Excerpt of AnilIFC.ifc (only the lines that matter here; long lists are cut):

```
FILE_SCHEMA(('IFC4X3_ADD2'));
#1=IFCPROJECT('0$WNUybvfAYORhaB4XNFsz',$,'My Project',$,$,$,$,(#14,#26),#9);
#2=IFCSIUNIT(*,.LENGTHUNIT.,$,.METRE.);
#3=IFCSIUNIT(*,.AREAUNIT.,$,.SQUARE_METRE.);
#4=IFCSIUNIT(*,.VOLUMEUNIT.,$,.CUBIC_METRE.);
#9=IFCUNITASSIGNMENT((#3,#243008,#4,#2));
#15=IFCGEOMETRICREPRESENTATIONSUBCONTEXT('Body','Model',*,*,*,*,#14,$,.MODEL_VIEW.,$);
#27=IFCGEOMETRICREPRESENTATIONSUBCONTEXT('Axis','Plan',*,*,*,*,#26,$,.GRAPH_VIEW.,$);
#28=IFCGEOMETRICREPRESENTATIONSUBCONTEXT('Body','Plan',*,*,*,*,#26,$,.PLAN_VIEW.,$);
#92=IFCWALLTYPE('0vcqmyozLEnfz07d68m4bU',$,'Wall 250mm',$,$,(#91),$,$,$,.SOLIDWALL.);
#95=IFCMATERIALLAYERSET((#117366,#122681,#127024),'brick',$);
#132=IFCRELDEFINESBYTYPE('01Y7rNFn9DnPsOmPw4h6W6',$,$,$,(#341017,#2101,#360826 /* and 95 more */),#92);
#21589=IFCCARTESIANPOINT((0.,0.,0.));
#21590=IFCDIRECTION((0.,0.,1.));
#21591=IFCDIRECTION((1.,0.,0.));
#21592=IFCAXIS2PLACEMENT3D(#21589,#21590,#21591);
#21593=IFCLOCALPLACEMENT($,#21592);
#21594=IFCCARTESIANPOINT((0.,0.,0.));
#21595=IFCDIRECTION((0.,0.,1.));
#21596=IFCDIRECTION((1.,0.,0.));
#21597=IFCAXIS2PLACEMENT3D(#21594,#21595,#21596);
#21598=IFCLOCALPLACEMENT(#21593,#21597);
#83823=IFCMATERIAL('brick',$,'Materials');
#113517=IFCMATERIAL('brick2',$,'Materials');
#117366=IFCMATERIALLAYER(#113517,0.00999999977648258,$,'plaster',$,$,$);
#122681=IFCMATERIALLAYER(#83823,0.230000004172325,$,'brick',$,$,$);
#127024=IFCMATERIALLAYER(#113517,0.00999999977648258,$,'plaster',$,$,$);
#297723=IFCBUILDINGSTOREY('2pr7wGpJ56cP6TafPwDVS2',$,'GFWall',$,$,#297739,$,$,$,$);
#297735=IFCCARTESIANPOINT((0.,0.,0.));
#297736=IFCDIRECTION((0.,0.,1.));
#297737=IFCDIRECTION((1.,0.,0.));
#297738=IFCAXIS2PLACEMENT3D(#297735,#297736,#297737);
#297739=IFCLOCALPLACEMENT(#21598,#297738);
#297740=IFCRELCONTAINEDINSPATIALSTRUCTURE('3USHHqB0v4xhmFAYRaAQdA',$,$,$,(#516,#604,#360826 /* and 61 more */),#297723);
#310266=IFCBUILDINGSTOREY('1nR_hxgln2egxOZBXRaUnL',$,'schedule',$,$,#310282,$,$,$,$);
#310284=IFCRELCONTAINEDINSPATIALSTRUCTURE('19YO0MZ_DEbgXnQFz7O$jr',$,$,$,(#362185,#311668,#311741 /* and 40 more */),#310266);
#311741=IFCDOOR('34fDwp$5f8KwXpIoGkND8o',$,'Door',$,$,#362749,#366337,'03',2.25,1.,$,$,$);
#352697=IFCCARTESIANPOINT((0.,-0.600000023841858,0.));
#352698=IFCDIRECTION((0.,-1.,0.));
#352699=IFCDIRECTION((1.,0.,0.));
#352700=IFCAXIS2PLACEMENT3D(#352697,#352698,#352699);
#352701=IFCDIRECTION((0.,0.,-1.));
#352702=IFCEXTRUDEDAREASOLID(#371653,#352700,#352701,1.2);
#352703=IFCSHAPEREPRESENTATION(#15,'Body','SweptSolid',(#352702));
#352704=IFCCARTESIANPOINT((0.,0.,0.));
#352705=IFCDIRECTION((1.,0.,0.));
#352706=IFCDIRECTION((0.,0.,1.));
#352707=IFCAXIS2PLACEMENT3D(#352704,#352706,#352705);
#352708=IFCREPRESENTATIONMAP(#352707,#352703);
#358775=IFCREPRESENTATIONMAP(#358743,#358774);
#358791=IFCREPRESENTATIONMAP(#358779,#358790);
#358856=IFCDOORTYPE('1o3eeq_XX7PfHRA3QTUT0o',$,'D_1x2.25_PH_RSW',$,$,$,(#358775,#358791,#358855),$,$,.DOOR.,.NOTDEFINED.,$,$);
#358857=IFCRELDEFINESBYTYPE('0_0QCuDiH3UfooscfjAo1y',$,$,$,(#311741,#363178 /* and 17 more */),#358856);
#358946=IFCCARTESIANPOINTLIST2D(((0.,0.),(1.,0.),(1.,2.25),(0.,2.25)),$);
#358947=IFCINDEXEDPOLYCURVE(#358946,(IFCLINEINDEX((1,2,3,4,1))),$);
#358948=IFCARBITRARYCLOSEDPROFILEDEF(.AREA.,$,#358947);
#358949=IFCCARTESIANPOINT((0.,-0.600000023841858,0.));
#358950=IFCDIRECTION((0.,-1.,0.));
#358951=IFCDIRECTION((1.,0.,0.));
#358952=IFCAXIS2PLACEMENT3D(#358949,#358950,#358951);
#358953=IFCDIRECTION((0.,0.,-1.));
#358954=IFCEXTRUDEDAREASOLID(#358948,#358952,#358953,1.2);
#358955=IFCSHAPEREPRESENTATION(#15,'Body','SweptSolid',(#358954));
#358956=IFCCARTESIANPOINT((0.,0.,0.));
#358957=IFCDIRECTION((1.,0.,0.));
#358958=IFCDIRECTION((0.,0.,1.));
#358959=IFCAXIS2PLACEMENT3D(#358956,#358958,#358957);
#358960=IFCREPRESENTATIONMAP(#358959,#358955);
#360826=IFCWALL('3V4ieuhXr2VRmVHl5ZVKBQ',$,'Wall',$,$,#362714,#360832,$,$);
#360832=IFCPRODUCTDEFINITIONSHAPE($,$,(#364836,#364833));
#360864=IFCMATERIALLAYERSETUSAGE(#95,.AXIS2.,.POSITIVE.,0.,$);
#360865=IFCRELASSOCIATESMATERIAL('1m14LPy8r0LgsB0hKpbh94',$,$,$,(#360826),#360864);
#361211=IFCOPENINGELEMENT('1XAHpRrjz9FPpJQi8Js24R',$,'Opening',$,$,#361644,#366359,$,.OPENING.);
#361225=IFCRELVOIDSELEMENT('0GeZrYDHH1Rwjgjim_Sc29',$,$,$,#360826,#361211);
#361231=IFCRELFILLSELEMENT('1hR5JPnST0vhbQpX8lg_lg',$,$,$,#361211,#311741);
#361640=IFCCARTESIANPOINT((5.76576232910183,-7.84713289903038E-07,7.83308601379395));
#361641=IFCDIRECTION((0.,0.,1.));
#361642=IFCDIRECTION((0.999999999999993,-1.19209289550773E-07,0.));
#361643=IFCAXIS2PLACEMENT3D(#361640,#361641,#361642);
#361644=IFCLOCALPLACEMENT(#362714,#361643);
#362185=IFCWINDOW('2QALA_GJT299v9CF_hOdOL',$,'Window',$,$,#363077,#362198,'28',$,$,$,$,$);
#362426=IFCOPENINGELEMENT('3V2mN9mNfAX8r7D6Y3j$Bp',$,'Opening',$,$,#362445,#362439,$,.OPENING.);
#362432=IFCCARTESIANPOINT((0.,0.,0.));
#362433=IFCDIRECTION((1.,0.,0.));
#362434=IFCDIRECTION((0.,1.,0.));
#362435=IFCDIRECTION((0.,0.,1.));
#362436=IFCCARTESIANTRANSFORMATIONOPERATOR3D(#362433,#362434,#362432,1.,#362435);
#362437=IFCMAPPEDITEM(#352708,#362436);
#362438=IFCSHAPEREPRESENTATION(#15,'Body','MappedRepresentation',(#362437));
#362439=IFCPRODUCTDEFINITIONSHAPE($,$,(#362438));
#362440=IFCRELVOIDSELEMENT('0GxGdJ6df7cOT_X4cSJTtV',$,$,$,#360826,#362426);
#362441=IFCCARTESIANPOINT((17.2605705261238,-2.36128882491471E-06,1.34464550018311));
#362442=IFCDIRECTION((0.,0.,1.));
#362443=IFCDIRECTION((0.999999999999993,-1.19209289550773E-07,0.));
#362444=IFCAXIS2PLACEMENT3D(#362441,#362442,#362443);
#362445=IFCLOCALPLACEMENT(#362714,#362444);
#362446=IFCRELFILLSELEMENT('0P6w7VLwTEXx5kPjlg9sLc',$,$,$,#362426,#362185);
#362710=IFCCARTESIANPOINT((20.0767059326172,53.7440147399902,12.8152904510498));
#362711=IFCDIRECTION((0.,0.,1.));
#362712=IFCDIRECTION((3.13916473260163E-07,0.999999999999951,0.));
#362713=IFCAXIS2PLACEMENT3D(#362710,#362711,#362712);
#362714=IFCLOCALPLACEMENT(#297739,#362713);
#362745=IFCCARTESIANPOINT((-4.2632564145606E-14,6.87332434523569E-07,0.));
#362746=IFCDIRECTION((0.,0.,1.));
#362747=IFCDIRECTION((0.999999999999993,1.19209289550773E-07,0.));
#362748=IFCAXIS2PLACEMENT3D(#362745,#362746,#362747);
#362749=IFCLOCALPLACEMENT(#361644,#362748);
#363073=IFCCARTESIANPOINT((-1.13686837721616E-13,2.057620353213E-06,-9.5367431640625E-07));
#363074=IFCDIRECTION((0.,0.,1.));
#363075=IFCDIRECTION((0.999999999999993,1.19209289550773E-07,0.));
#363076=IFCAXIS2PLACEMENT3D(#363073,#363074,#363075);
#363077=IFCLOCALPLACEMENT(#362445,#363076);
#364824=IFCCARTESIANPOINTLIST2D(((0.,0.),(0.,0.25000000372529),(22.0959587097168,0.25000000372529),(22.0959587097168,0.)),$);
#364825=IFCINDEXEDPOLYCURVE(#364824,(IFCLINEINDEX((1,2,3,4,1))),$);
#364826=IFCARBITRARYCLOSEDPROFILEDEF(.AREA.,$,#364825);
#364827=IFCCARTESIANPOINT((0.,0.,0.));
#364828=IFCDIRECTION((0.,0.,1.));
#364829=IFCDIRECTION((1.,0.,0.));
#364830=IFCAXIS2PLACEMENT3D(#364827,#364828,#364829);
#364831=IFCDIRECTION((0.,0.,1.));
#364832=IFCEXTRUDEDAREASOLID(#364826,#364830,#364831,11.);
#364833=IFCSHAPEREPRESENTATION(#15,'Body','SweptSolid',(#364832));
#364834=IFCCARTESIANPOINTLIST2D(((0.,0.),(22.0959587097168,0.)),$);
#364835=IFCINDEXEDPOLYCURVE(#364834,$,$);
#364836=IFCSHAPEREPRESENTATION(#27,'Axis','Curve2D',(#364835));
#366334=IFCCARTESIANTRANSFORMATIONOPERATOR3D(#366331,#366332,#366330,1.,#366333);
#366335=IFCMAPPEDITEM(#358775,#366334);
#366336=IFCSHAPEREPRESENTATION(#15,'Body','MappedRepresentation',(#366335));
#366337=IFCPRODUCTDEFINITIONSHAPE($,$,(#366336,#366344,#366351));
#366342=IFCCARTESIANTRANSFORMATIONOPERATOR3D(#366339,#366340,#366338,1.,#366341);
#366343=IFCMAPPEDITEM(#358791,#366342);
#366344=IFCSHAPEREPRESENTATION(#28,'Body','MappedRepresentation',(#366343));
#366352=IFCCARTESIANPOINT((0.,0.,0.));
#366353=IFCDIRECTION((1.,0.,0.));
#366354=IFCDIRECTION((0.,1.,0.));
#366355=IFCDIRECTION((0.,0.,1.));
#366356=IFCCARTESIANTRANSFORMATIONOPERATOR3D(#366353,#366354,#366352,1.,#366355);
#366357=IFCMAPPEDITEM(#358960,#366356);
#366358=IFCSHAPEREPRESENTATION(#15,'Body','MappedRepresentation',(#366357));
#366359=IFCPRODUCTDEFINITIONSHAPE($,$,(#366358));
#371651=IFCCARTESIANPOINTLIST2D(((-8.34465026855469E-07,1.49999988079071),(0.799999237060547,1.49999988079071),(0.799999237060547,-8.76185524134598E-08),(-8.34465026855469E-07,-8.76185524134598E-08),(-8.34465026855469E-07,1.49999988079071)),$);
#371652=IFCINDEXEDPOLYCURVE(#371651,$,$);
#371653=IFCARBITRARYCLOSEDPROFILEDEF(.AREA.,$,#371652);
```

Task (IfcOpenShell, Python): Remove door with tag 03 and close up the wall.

```python
import ifcopenshell
import ifcopenshell.api.feature
import ifcopenshell.api.root
import ifcopenshell.geom
import ifcopenshell.util.shape

model = ifcopenshell.open("AnilIFC.ifc")
settings = ifcopenshell.geom.settings()


def volume(element):
    """Net volume in cubic metres, openings subtracted."""
    shape = ifcopenshell.geom.create_shape(settings, element)
    return ifcopenshell.util.shape.get_volume(shape.geometry)


door = model.by_guid("34fDwp$5f8KwXpIoGkND8o")
opening = door.FillsVoids[0].RelatingOpeningElement
wall = opening.VoidsElements[0].RelatingBuildingElement
before = volume(wall)

ifcopenshell.api.root.remove_product(model, product=door)
ifcopenshell.api.feature.remove_feature(model, feature=opening)

after = volume(wall)

print(f"wall volume {before:.3f} -> {after:.3f} m3")

model.write("AnilIFC_updated.ifc")
```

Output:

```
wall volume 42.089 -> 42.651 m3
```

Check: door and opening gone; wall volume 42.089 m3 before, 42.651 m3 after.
